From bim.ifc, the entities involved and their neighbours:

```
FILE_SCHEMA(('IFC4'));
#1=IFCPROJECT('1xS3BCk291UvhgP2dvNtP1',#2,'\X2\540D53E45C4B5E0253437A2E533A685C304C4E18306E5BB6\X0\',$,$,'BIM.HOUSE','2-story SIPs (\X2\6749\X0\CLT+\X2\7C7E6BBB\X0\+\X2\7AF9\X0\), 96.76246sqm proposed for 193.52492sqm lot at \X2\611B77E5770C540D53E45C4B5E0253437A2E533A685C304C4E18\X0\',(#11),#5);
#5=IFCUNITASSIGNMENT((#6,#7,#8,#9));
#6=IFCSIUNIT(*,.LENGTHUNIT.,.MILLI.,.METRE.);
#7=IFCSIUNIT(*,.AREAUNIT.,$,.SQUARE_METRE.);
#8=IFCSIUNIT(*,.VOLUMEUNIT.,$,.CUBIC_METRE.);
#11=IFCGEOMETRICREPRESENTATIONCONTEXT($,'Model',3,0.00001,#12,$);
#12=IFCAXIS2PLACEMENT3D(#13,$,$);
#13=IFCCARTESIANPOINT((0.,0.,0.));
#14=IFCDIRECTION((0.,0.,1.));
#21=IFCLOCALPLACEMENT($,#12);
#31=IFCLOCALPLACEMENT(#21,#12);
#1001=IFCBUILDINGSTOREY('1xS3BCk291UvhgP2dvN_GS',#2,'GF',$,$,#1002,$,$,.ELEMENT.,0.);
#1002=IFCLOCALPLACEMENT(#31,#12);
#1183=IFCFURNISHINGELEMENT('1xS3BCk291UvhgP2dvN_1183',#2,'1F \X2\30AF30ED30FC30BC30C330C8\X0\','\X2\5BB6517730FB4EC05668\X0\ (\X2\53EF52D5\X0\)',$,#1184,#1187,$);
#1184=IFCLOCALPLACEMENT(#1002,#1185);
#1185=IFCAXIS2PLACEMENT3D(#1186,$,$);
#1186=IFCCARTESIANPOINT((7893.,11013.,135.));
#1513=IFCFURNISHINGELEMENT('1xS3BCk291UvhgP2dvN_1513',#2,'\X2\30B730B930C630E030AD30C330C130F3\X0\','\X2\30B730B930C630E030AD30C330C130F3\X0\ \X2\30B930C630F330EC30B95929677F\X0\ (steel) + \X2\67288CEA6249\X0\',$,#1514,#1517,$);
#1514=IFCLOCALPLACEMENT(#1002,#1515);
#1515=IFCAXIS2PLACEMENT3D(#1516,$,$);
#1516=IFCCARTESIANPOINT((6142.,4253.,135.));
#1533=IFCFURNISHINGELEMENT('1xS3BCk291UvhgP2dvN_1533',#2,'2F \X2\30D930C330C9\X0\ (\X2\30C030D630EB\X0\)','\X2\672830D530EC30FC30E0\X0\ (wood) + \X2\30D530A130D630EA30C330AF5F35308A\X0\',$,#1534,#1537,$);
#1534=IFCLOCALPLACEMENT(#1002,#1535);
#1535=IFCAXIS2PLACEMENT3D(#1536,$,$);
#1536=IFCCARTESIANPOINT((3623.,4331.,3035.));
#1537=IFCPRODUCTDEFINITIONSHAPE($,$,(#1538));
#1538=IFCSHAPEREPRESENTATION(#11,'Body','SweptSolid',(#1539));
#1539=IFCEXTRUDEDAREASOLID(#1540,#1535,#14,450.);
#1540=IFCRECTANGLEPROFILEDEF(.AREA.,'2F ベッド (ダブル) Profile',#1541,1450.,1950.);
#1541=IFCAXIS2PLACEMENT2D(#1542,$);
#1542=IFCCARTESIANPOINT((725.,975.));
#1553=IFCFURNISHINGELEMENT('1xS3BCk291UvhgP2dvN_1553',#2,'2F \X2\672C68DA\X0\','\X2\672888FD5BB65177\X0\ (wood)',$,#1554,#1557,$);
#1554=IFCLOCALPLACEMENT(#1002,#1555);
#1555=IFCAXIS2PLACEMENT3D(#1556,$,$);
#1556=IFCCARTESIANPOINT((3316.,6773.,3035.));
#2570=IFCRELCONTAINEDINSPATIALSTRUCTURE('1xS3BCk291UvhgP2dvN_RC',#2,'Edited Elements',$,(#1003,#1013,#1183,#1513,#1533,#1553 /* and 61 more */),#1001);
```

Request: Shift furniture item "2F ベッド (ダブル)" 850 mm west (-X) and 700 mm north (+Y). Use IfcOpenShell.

```python
import ifcopenshell
import ifcopenshell.api.geometry
import ifcopenshell.util.placement
import ifcopenshell.util.unit

model = ifcopenshell.open("bim.ifc")
unit_scale = ifcopenshell.util.unit.calculate_unit_scale(model)

item = model.by_guid("1xS3BCk291UvhgP2dvN_1533")
matrix = ifcopenshell.util.placement.get_local_placement(item.ObjectPlacement)
matrix[0, 3] -= 0.85 / unit_scale
matrix[1, 3] += 0.7 / unit_scale
ifcopenshell.api.geometry.edit_object_placement(model, product=item, matrix=matrix, is_si=False)

print(ifcopenshell.util.placement.get_local_placement(item.ObjectPlacement).round(3) + 0.0)

model.write("bim_rev.ifc")
```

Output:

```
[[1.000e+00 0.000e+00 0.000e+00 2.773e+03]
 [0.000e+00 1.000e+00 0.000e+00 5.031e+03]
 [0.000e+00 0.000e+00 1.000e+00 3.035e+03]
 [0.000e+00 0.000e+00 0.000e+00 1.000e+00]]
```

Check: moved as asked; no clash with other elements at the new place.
